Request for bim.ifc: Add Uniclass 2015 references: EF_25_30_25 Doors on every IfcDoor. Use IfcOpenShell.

First a look at what the model holds.

```python
import ifcopenshell

model = ifcopenshell.open("bim.ifc")
print(model.schema)
print("classifications:", [c.Name for c in model.by_type("IfcClassification")])
for ifc_class in ("IfcDoor", "IfcRoof", "IfcStair", "IfcWall", "IfcWindow"):
    print(ifc_class, len(model.by_type(ifc_class)))
```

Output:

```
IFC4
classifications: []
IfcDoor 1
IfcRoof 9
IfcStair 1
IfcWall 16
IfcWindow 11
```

```python
import ifcopenshell
import ifcopenshell.api.classification

model = ifcopenshell.open("bim.ifc")

system = ifcopenshell.api.classification.add_classification(model, classification="Uniclass 2015")

codes = {
    "IfcDoor": ("EF_25_30_25", "Doors"),
}
for ifc_class, (code, name) in codes.items():
    products = model.by_type(ifc_class)
    ifcopenshell.api.classification.add_reference(
        model, products=products, classification=system, identification=code, name=name
    )
    print(code, len(products))

model.write("bim_rev.ifc")
```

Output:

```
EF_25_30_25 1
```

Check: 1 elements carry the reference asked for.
